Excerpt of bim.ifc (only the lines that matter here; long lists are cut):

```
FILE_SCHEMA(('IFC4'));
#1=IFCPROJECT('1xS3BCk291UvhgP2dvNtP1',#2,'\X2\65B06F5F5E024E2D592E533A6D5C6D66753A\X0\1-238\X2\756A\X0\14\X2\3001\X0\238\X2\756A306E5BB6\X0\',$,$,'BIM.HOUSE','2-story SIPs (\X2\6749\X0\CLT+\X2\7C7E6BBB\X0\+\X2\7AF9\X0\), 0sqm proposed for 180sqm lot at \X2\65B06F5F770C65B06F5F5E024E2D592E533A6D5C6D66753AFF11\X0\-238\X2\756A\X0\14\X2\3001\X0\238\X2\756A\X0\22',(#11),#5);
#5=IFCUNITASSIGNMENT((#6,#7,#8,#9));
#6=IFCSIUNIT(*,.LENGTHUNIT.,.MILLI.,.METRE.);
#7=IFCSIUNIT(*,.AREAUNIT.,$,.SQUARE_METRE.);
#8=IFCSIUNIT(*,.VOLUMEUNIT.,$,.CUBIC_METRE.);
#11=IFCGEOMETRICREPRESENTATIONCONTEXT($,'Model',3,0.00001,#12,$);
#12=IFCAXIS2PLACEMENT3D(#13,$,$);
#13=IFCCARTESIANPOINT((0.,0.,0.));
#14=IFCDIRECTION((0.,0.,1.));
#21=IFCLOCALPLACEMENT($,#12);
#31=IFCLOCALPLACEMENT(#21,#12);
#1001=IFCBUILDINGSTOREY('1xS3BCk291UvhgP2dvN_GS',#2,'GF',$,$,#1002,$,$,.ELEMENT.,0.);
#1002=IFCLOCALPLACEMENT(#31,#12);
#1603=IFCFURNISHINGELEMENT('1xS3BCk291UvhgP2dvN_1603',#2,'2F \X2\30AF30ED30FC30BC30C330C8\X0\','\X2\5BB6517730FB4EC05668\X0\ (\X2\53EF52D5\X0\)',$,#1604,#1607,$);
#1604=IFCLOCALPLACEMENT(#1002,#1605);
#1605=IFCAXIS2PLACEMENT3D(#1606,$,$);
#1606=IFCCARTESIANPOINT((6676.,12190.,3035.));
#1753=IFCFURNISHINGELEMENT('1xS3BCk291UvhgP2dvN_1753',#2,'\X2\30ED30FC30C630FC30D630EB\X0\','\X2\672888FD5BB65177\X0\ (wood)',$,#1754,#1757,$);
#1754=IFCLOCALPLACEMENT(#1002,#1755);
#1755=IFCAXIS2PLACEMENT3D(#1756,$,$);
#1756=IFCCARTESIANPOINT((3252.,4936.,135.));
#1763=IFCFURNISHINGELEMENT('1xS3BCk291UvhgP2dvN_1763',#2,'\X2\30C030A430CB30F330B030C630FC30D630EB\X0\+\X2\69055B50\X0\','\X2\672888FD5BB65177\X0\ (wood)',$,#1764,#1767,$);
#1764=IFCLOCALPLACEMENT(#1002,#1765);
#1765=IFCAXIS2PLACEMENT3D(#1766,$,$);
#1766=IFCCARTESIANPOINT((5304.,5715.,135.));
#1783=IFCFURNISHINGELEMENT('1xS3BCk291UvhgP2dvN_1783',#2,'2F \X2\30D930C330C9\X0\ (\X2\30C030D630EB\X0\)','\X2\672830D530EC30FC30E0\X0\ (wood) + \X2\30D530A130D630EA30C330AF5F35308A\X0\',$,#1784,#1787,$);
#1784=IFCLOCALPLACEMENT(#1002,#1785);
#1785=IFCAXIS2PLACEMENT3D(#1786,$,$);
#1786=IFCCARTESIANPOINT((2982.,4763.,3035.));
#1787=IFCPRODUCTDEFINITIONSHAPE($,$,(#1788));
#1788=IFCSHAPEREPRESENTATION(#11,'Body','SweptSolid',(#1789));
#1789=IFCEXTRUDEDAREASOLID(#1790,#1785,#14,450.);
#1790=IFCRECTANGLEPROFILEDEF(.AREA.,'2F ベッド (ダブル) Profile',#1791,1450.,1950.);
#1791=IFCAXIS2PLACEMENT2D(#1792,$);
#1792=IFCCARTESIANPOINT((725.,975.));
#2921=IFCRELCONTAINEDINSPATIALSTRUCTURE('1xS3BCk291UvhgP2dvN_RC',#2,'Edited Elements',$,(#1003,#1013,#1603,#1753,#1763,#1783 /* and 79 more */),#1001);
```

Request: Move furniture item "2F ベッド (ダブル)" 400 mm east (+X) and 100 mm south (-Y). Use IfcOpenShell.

```python
import ifcopenshell
import ifcopenshell.api.geometry
import ifcopenshell.util.placement
import ifcopenshell.util.unit

model = ifcopenshell.open("bim.ifc")
unit_scale = ifcopenshell.util.unit.calculate_unit_scale(model)

item = model.by_id(1783)
matrix = ifcopenshell.util.placement.get_local_placement(item.ObjectPlacement)
matrix[0, 3] += 0.4 / unit_scale
matrix[1, 3] -= 0.1 / unit_scale
ifcopenshell.api.geometry.edit_object_placement(model, product=item, matrix=matrix, is_si=False)

print(ifcopenshell.util.placement.get_local_placement(item.ObjectPlacement).round(3) + 0.0)

model.write("bim_v2.ifc")
```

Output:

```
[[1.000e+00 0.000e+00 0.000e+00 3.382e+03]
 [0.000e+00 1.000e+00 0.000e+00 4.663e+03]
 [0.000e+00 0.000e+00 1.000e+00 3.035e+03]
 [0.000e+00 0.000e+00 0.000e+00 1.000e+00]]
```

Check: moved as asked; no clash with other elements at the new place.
